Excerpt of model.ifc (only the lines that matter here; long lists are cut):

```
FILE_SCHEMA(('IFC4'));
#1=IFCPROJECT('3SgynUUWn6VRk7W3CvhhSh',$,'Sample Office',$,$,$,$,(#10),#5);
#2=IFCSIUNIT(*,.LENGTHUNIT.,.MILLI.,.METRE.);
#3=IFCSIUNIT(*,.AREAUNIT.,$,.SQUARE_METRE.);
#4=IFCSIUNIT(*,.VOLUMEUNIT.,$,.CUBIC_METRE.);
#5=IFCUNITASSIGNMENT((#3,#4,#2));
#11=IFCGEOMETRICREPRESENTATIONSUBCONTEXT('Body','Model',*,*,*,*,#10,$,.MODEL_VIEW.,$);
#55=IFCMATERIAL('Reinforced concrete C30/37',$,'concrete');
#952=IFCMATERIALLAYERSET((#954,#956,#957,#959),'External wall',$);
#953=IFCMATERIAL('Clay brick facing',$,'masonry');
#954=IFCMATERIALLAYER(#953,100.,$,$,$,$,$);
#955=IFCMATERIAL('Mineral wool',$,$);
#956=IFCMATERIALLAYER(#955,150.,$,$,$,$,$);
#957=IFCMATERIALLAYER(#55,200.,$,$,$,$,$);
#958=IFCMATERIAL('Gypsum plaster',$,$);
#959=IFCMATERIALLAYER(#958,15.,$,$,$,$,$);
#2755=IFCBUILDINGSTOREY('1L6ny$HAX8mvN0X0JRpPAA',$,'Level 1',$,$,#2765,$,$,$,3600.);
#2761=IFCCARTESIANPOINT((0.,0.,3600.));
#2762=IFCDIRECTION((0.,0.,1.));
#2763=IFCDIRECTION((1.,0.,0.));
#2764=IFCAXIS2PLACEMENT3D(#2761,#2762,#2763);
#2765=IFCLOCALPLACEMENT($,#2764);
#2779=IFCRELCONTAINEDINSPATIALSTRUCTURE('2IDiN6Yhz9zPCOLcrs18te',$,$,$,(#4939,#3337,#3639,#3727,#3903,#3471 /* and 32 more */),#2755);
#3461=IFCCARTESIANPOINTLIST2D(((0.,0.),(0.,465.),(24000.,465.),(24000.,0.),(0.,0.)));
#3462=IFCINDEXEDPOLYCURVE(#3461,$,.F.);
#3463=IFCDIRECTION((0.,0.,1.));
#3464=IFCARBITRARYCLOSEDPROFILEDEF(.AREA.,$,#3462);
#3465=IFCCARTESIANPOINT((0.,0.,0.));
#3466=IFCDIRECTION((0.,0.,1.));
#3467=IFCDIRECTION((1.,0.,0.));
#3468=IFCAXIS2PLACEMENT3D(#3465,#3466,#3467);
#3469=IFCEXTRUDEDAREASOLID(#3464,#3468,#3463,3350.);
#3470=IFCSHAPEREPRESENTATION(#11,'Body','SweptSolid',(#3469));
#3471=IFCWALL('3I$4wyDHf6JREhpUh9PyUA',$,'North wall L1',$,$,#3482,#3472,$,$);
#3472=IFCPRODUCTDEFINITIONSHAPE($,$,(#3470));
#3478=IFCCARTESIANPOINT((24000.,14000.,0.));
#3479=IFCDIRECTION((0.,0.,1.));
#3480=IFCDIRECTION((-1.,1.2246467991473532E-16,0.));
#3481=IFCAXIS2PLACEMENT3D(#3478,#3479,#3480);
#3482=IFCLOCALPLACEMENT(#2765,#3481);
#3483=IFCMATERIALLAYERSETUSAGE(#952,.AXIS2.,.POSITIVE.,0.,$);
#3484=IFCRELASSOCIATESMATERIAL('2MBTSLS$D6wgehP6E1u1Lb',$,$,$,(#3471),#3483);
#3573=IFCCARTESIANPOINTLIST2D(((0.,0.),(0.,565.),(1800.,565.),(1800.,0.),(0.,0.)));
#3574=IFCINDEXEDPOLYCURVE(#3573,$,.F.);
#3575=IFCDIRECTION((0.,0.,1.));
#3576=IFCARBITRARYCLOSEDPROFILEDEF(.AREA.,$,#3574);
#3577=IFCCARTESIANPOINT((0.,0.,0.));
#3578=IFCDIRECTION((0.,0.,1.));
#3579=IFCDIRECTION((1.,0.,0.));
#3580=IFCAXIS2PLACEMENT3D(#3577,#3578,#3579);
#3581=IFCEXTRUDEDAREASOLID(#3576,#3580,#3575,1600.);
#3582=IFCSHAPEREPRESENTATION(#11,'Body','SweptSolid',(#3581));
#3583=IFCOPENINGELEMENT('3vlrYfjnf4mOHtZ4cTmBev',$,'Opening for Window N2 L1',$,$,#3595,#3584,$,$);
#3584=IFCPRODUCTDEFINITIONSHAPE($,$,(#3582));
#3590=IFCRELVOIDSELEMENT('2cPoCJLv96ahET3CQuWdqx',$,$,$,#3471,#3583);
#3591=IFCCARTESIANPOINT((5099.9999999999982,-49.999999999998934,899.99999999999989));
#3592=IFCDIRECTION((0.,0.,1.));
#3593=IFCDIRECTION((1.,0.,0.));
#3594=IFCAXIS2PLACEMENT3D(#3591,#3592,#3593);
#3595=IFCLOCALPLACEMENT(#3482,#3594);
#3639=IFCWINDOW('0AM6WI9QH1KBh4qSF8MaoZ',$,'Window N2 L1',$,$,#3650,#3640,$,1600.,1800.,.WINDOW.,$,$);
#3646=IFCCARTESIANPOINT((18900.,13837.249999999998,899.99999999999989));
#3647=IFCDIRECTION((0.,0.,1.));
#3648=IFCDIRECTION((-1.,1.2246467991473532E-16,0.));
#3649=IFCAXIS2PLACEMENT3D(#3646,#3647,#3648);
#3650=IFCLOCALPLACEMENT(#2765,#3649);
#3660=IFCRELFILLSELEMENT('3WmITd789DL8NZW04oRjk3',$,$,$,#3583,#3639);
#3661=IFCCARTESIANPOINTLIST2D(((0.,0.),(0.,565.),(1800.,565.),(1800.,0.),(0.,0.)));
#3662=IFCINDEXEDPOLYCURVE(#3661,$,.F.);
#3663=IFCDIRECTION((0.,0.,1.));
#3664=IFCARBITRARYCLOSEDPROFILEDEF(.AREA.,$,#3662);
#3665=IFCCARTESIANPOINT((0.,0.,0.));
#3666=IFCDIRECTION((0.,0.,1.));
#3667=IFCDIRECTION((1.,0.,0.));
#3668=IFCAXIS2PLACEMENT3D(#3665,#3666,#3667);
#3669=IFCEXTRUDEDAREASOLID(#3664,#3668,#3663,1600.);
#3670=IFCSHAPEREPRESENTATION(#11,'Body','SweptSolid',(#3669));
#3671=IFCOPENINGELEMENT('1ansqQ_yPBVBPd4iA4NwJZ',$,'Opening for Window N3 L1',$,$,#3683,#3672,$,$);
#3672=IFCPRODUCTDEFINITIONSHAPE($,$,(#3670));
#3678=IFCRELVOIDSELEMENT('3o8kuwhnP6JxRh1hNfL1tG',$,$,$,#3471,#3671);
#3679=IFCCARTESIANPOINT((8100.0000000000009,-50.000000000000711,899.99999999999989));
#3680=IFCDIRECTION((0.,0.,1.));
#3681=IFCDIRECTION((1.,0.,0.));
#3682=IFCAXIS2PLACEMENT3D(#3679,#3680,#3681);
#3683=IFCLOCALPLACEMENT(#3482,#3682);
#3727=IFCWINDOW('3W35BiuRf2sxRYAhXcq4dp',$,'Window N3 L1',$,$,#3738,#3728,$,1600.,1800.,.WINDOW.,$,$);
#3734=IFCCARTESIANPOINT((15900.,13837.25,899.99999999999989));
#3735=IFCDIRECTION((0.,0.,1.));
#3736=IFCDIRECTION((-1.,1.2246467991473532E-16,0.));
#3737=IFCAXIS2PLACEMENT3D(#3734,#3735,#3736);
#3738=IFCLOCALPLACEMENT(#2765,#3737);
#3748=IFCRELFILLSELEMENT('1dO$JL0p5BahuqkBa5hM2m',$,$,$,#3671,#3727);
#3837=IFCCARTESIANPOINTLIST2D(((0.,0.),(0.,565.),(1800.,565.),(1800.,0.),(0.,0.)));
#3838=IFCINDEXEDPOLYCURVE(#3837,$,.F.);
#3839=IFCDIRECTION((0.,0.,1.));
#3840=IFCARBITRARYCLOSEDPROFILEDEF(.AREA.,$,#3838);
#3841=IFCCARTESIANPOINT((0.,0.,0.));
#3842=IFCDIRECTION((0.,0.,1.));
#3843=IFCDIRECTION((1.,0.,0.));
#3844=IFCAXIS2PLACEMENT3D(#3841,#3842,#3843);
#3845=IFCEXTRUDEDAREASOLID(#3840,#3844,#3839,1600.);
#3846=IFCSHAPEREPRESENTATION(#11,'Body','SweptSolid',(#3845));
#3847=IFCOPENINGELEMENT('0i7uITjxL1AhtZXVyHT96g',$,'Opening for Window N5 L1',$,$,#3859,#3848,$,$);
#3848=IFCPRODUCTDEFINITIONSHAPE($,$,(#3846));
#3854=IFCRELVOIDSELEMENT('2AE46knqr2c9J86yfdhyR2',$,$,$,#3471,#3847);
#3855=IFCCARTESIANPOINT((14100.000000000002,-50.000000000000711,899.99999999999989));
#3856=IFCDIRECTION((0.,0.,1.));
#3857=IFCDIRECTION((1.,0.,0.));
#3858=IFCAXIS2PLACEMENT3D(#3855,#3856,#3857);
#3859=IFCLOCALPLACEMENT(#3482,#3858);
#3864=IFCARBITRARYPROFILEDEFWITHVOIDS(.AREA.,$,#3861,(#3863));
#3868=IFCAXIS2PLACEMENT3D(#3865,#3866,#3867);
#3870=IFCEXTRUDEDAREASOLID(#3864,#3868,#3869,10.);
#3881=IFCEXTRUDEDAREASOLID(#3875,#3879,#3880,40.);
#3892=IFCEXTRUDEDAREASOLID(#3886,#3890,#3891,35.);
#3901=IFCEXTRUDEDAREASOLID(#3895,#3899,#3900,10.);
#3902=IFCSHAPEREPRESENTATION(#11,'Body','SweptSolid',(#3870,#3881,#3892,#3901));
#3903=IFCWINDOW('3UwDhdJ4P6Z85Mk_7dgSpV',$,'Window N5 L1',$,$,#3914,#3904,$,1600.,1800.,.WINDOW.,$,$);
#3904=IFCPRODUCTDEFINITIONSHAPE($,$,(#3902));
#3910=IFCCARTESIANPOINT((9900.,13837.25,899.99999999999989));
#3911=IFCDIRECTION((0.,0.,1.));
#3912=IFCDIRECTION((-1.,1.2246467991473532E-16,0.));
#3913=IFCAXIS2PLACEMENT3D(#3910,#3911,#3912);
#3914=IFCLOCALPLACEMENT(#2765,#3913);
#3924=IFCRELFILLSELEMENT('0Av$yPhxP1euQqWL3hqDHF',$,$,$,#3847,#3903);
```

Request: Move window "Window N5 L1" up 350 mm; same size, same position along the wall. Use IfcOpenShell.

```python
import numpy as np
import ifcopenshell
import ifcopenshell.api.geometry
import ifcopenshell.util.placement
import ifcopenshell.util.unit

model = ifcopenshell.open("model.ifc")
unit_scale = ifcopenshell.util.unit.calculate_unit_scale(model)

window = model.by_guid("3UwDhdJ4P6Z85Mk_7dgSpV")
opening = window.FillsVoids[0].RelatingOpeningElement
dz = 350.0

shift = np.array([0.0, 0.0, dz])
# The window is not placed relative to its opening, so move both.
for product in (opening, window):
    matrix = ifcopenshell.util.placement.get_local_placement(product.ObjectPlacement)
    matrix[:3, 3] += shift
    ifcopenshell.api.geometry.edit_object_placement(model, product=product, matrix=matrix, is_si=False)

print(f"moved by {dz * unit_scale:+.3f} m")

model.write("model_edited.ifc")
```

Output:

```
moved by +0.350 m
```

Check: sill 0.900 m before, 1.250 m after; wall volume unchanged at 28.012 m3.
